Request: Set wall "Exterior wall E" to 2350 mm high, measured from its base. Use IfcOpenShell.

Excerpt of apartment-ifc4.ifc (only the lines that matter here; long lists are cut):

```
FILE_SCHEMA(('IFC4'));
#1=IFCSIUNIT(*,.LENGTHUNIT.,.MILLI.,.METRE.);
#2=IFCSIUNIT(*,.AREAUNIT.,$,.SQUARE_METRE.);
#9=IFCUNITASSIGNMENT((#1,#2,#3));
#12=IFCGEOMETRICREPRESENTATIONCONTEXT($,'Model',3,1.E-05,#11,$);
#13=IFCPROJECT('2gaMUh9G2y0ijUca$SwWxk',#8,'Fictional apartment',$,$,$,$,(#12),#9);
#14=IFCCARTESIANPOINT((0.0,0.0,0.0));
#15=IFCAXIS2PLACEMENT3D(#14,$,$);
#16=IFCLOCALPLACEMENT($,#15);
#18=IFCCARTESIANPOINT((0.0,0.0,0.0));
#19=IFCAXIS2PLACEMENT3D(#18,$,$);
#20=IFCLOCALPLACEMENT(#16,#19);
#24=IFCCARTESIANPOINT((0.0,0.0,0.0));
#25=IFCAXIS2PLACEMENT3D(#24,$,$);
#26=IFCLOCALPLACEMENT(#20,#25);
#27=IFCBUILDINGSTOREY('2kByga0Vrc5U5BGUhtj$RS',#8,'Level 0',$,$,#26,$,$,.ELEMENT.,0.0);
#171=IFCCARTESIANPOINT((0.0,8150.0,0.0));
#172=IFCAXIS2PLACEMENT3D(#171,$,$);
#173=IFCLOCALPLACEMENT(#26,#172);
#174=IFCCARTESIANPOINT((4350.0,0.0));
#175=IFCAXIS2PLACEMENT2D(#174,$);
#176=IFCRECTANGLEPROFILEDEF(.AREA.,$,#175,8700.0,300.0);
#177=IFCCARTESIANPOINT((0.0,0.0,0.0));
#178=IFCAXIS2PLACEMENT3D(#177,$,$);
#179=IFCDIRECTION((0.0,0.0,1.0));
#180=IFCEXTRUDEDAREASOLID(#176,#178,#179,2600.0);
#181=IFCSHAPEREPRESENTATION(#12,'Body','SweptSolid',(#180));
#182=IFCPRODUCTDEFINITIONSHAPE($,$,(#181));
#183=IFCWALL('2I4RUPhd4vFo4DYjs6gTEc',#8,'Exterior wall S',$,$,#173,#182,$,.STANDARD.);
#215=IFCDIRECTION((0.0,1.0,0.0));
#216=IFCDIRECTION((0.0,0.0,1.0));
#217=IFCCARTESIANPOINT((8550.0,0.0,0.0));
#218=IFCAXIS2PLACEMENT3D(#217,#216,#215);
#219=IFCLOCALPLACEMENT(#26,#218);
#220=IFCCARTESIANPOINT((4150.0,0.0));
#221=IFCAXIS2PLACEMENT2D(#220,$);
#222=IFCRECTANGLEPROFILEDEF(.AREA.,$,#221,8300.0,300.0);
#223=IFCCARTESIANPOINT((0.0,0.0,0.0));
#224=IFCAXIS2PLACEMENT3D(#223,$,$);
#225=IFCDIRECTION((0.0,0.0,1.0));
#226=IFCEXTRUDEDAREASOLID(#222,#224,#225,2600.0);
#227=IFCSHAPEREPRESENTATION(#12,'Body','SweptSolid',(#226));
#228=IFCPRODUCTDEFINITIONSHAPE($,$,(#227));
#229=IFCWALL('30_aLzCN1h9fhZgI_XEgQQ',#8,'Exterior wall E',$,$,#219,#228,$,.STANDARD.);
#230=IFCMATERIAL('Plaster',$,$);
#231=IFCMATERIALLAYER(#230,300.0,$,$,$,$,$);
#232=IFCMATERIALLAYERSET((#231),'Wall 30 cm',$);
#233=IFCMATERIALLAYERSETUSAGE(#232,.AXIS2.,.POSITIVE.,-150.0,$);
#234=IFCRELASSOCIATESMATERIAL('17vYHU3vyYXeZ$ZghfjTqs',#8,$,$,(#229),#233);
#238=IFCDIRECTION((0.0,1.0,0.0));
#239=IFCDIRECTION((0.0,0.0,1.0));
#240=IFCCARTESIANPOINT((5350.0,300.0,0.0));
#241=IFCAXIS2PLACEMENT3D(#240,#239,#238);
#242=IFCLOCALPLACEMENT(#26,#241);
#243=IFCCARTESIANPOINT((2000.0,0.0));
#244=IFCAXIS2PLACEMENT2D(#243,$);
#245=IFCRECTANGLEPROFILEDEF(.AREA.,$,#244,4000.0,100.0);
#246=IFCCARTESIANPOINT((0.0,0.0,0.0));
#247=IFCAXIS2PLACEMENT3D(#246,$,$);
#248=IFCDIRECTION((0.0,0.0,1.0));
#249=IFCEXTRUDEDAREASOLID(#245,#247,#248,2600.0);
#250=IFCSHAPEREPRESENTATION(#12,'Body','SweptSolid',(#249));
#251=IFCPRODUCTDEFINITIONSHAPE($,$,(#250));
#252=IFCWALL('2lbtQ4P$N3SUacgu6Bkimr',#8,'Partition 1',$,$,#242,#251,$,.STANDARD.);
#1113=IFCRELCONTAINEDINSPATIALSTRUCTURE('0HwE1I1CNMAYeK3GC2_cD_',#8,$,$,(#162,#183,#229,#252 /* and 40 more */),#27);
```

```python
import ifcopenshell
import ifcopenshell.geom
import ifcopenshell.util.shape

model = ifcopenshell.open("apartment-ifc4.ifc")
settings = ifcopenshell.geom.settings()


def volume(element):
    """Net volume in cubic metres, openings subtracted."""
    shape = ifcopenshell.geom.create_shape(settings, element)
    return ifcopenshell.util.shape.get_volume(shape.geometry)


wall = model.by_guid("30_aLzCN1h9fhZgI_XEgQQ")
before = volume(wall)

body = next(r for r in wall.Representation.Representations if r.RepresentationIdentifier == "Body")
solid = body.Items[0]
old_height = solid.Depth
solid.Depth = 2350.0
after = volume(wall)

print(f"height {old_height:g} -> {solid.Depth:g}, volume {before:.3f} -> {after:.3f} m3")

model.write("apartment-ifc4_rev.ifc")
```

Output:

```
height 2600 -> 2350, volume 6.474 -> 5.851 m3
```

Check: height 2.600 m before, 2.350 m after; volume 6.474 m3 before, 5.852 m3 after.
